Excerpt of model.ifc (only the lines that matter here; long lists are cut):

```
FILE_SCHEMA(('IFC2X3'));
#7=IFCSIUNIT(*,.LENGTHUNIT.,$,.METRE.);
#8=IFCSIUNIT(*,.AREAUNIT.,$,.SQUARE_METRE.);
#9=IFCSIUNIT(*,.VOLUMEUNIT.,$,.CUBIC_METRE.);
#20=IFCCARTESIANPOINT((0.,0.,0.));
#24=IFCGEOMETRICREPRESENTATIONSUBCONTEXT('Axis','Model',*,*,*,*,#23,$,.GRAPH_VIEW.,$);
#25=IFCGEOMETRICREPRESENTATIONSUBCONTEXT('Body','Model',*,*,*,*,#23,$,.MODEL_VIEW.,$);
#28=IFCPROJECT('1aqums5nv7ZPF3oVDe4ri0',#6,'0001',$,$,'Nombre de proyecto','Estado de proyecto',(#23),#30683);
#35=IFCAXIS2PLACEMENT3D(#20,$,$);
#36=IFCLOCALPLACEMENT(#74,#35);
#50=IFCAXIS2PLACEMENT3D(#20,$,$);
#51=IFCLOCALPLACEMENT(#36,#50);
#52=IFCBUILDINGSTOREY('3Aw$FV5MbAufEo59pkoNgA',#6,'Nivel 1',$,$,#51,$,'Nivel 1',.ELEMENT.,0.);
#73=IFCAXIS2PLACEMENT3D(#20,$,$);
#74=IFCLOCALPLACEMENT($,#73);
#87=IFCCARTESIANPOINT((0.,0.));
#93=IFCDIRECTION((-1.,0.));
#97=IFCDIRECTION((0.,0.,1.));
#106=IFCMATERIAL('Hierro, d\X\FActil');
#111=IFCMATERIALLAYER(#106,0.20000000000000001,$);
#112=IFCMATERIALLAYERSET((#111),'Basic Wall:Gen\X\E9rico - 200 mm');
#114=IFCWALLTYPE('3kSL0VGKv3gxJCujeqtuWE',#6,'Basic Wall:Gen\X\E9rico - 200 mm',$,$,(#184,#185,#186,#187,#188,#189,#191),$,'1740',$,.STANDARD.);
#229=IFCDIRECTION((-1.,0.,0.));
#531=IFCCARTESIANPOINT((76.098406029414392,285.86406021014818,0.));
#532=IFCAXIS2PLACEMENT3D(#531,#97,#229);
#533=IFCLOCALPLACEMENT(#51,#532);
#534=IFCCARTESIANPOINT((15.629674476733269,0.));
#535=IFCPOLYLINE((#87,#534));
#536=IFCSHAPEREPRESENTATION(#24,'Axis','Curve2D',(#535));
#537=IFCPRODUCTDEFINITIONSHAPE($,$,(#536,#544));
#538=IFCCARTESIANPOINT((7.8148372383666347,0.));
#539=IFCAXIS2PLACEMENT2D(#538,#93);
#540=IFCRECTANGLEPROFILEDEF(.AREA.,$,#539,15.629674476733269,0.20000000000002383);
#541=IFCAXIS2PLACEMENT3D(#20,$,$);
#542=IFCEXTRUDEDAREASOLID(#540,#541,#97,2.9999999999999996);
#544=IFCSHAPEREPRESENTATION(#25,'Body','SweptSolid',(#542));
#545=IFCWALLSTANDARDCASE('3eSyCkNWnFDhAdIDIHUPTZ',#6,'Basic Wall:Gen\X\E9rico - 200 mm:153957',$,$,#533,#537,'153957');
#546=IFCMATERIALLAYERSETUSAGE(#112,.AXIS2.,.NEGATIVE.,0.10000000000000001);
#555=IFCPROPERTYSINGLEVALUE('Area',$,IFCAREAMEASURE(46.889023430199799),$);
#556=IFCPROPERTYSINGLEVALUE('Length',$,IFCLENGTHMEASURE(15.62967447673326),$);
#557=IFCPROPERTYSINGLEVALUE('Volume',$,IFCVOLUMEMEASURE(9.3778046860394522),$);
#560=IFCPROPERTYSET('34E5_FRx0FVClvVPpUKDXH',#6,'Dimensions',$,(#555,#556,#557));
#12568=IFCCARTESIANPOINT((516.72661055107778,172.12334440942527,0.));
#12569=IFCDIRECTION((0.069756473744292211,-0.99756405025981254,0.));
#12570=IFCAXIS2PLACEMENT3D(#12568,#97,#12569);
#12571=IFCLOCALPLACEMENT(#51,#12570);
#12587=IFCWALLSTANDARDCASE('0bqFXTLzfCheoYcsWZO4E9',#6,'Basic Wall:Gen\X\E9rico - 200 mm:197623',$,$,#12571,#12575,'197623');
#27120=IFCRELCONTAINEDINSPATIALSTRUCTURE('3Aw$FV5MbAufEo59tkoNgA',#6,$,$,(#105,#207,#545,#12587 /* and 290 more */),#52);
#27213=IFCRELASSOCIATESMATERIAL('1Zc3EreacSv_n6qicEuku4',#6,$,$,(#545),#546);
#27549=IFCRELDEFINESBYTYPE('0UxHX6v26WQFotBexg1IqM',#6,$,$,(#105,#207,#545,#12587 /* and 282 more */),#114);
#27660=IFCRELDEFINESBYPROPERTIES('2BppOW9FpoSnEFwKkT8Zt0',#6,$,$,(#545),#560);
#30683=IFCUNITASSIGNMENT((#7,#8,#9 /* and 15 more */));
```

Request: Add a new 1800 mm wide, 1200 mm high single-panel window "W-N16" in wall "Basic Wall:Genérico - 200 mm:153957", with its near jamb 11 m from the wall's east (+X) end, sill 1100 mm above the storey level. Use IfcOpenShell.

```python
import numpy as np
import ifcopenshell
import ifcopenshell.api.feature
import ifcopenshell.api.geometry
import ifcopenshell.api.pset
import ifcopenshell.api.root
import ifcopenshell.api.spatial
import ifcopenshell.api.type
import ifcopenshell.geom
import ifcopenshell.util.element
import ifcopenshell.util.placement
import ifcopenshell.util.representation
import ifcopenshell.util.shape
import ifcopenshell.util.unit

model = ifcopenshell.open("model.ifc")
unit_scale = ifcopenshell.util.unit.calculate_unit_scale(model)
area_scale = ifcopenshell.util.unit.calculate_unit_scale(model, "AREAUNIT")
volume_scale = ifcopenshell.util.unit.calculate_unit_scale(model, "VOLUMEUNIT")
settings = ifcopenshell.geom.settings()


def volume(element):
    """Net volume in cubic metres, openings subtracted."""
    shape = ifcopenshell.geom.create_shape(settings, element)
    return ifcopenshell.util.shape.get_volume(shape.geometry)


wall = model.by_guid("3eSyCkNWnFDhAdIDIHUPTZ")
storey = ifcopenshell.util.element.get_container(wall, ifc_class="IfcBuildingStorey")
context = ifcopenshell.util.representation.get_context(model, "Model", "Body", "MODEL_VIEW")
before = volume(wall)

width, height, from_end, sill = 1.8, 1.2, 11, 1.1  # metres

# The wall runs along its own X axis, and the end named is its -X end.
wall_shape = ifcopenshell.geom.create_shape(settings, wall)
x, y, z = ifcopenshell.util.shape.get_vertices(wall_shape.geometry).T
start = x.min() + from_end
face, thickness = float(y.min()), float(y.max() - y.min())
wall_matrix = ifcopenshell.util.placement.get_local_placement(wall.ObjectPlacement)
level = ifcopenshell.util.placement.get_local_placement(storey.ObjectPlacement)[2, 3]


def in_wall(x, y):
    """Placement at x, y metres in the wall's axes, at sill height."""
    matrix = wall_matrix.copy()
    matrix[:, 3] = wall_matrix @ np.array([x / unit_scale, y / unit_scale, 0.0, 1.0])
    matrix[2, 3] = level + sill / unit_scale
    return matrix


# Opening: a box that overshoots both wall faces by 50 mm.
opening = ifcopenshell.api.root.create_entity(model, ifc_class="IfcOpeningElement")
box = ifcopenshell.api.geometry.add_wall_representation(
    model, context=context, length=width, height=height, thickness=thickness + 0.1
)
ifcopenshell.api.geometry.assign_representation(model, product=opening, representation=box)
ifcopenshell.api.geometry.edit_object_placement(model, product=opening, matrix=in_wall(start, face - 0.05), is_si=False)
ifcopenshell.api.feature.add_feature(model, feature=opening, element=wall)

window = ifcopenshell.api.root.create_entity(model, ifc_class="IfcWindow", name="W-N16")
window.OverallWidth, window.OverallHeight = width / unit_scale, height / unit_scale
body = ifcopenshell.api.geometry.add_window_representation(
    model,
    context=context,
    overall_width=window.OverallWidth,
    overall_height=window.OverallHeight,
    partition_type="SINGLE_PANEL",
)
ifcopenshell.api.geometry.assign_representation(model, product=window, representation=body)
ifcopenshell.api.spatial.assign_container(model, products=[window], relating_structure=storey)
fills = ifcopenshell.api.feature.add_filling(model, opening=opening, element=window)
fills.OwnerHistory = window.OwnerHistory  # required in IFC2X3

# IFC2X3 keeps the operation on the window style.
style = ifcopenshell.api.root.create_entity(model, ifc_class="IfcWindowStyle", name="W-N16")
style.OperationType, style.ConstructionType = "SINGLE_PANEL", "NOTDEFINED"
style.ParameterTakesPrecedence = style.Sizeable = False
ifcopenshell.api.type.assign_type(model, related_objects=[window], relating_type=style)

# Centre the window in the wall's thickness.
ifcopenshell.api.geometry.edit_object_placement(model, product=window, matrix=in_wall(start, face), is_si=False)
window_shape = ifcopenshell.geom.create_shape(settings, window)
depth = ifcopenshell.util.shape.get_vertices(window_shape.geometry)[:, 1]
offset = face + thickness / 2 - (depth.min() + depth.max()) / 2
ifcopenshell.api.geometry.edit_object_placement(model, product=window, matrix=in_wall(start, offset), is_si=False)

after = volume(wall)

# Update the wall's stored quantities.
pset = model.by_id(ifcopenshell.util.element.get_pset(wall, "Dimensions", should_inherit=False)["id"])
ifcopenshell.api.pset.edit_pset(model, pset=pset, properties={
    "Area": model.create_entity("IfcAreaMeasure", after / thickness / area_scale),
    "Volume": model.create_entity("IfcVolumeMeasure", after / volume_scale),
})

print(f"wall volume {before:.3f} -> {after:.3f} m3")

model.write("model_edited.ifc")
```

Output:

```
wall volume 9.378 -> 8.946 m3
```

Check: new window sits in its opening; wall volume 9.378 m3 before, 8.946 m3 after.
